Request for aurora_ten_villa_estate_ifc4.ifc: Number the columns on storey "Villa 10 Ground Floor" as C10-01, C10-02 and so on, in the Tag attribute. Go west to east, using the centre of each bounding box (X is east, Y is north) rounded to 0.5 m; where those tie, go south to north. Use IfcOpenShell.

First a look at what the model holds.

```python
import ifcopenshell
import ifcopenshell.util.element
import ifcopenshell.util.placement

model = ifcopenshell.open("aurora_ten_villa_estate_ifc4.ifc")
print(model.schema)
storey = next(s for s in model.by_type("IfcBuildingStorey") if s.Name == "Villa 10 Ground Floor")
columns = [e for e in ifcopenshell.util.element.get_decomposition(storey) if e.is_a("IfcColumn")]
for e in sorted(columns, key=lambda e: e.id()):
    origin = ifcopenshell.util.placement.get_local_placement(e.ObjectPlacement)[:3, 3]
    print(e.id(), e.Tag, e.Name, origin.round(2) + 0.0, sep=" | ")
```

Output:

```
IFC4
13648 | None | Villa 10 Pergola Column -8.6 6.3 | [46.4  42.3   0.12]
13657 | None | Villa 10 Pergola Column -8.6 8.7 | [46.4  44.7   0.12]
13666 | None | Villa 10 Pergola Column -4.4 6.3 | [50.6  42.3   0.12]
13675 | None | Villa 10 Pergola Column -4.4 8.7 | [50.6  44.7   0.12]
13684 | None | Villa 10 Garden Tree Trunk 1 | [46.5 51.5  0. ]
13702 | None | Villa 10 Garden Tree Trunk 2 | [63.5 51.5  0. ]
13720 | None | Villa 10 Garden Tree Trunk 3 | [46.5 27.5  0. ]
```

```python
import ifcopenshell
import ifcopenshell.geom
import ifcopenshell.util.element
import ifcopenshell.util.shape

model = ifcopenshell.open("aurora_ten_villa_estate_ifc4.ifc")
settings = ifcopenshell.geom.settings()
settings.set("use-world-coords", True)


def centre(element):
    shape = ifcopenshell.geom.create_shape(settings, element)
    return ifcopenshell.util.shape.get_bbox_centroid(shape.geometry)


storey = next(s for s in model.by_type("IfcBuildingStorey") if s.Name == "Villa 10 Ground Floor")
columns = [e for e in ifcopenshell.util.element.get_decomposition(storey) if e.is_a("IfcColumn")]

# Insertion points can sit at a corner or the storey origin, so sort by the geometry (in metres).
centres = {e: centre(e) for e in columns}
columns.sort(key=lambda e: (round(centres[e][0] / 0.5), centres[e][1]))

for i, e in enumerate(columns, start=1):
    number = f"C10-{i:02d}"
    e.Tag = number
    print(e.id(), number)

model.write("aurora_ten_villa_estate_ifc4_rev.ifc")
```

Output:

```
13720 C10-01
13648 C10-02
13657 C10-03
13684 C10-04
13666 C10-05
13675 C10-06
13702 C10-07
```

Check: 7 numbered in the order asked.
